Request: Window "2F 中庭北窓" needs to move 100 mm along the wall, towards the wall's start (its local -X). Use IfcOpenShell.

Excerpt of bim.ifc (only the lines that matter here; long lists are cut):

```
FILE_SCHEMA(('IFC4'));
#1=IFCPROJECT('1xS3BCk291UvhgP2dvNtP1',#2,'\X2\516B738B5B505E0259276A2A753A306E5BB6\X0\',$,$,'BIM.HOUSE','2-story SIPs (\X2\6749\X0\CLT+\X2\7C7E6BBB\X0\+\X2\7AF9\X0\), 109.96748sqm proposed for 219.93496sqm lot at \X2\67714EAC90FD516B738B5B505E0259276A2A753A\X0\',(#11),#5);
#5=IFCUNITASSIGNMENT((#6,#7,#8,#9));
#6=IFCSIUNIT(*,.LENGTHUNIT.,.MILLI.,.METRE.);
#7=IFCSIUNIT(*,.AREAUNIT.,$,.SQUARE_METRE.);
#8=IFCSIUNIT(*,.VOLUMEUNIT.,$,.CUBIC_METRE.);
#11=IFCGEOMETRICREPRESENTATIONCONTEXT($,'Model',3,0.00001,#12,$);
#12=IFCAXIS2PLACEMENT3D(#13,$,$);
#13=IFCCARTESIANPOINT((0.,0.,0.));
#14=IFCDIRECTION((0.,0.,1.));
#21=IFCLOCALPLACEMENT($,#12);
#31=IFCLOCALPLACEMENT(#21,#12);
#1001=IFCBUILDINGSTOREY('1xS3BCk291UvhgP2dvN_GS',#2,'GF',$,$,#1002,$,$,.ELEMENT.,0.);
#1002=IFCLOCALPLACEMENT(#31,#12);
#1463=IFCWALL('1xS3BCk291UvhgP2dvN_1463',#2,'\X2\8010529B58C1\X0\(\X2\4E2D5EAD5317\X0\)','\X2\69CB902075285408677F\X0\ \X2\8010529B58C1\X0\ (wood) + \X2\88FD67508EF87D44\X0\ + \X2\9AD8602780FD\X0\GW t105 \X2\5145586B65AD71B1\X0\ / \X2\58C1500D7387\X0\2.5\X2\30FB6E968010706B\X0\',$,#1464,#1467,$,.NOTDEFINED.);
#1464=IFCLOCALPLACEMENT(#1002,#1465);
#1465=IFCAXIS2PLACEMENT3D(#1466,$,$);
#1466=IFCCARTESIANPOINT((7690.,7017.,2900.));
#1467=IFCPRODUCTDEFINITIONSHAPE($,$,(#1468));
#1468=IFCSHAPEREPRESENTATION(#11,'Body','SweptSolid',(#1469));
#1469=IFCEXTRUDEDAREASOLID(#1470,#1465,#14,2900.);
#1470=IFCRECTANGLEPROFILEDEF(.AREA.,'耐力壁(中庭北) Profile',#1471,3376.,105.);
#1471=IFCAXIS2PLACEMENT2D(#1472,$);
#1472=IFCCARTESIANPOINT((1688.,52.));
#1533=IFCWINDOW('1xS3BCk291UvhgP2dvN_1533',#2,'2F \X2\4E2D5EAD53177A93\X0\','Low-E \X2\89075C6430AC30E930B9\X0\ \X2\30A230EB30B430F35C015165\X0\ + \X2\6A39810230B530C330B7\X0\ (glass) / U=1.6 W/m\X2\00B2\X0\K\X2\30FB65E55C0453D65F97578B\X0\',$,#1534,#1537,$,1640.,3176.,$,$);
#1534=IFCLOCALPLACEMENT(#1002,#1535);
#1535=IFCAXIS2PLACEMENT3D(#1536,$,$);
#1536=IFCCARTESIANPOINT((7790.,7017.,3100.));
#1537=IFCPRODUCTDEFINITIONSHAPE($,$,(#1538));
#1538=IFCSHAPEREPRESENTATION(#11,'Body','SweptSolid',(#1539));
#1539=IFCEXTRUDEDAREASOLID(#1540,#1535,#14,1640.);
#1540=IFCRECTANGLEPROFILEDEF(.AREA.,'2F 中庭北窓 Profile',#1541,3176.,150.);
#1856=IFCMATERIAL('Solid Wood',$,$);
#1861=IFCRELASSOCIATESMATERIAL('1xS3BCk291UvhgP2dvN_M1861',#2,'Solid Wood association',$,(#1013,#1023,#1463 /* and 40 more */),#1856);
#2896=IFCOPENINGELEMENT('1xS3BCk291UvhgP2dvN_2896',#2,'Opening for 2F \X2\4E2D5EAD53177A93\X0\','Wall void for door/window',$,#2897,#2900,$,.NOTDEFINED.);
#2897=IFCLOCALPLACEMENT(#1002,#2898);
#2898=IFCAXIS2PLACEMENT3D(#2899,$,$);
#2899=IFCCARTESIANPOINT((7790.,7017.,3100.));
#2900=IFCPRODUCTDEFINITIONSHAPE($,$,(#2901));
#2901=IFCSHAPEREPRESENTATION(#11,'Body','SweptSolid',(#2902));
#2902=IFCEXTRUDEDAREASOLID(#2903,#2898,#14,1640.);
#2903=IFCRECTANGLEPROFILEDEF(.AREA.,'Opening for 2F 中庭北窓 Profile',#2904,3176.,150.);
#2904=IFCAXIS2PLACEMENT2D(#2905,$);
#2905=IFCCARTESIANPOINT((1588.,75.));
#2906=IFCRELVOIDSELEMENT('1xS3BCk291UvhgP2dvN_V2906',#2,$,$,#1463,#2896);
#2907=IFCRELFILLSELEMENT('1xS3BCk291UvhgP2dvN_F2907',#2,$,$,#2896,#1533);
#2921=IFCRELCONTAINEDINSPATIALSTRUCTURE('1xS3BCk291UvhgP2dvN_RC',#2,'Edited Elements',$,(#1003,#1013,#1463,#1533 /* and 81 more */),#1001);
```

```python
import ifcopenshell
import ifcopenshell.api.geometry
import ifcopenshell.util.placement

model = ifcopenshell.open("bim.ifc")

window = model.by_guid("1xS3BCk291UvhgP2dvN_1533")
opening = window.FillsVoids[0].RelatingOpeningElement
wall = opening.VoidsElements[0].RelatingBuildingElement

wall_matrix = ifcopenshell.util.placement.get_local_placement(wall.ObjectPlacement)
shift = wall_matrix[:3, 0] * -100.0
before = ifcopenshell.util.placement.get_local_placement(window.ObjectPlacement)[:3, 3].copy()

# The window is not placed relative to its opening, so move both.
for product in (opening, window):
    matrix = ifcopenshell.util.placement.get_local_placement(product.ObjectPlacement)
    matrix[:3, 3] += shift
    ifcopenshell.api.geometry.edit_object_placement(model, product=product, matrix=matrix, is_si=False)

after = ifcopenshell.util.placement.get_local_placement(window.ObjectPlacement)[:3, 3]
print("window moved by", (after - before).round(3) + 0.0)

model.write("bim_updated.ifc")
```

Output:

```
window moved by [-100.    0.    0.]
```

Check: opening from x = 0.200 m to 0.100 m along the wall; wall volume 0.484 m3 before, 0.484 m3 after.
